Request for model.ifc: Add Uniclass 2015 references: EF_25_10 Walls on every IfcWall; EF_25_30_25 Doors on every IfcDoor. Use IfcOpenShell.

First a look at what the model holds.

```python
import ifcopenshell

model = ifcopenshell.open("model.ifc")
print(model.schema)
print("classifications:", [c.Name for c in model.by_type("IfcClassification")])
for ifc_class in ("IfcDoor", "IfcRoof", "IfcStair", "IfcWall", "IfcWindow"):
    print(ifc_class, len(model.by_type(ifc_class)))
```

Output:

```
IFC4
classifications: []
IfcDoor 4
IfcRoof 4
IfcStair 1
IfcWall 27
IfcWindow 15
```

```python
import ifcopenshell
import ifcopenshell.api.classification

model = ifcopenshell.open("model.ifc")

system = ifcopenshell.api.classification.add_classification(model, classification="Uniclass 2015")

codes = {
    "IfcWall": ("EF_25_10", "Walls"),
    "IfcDoor": ("EF_25_30_25", "Doors"),
}
for ifc_class, (code, name) in codes.items():
    products = model.by_type(ifc_class)
    ifcopenshell.api.classification.add_reference(
        model, products=products, classification=system, identification=code, name=name
    )
    print(code, len(products))

model.write("model_edited.ifc")
```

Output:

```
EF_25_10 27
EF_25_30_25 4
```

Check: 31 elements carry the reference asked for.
